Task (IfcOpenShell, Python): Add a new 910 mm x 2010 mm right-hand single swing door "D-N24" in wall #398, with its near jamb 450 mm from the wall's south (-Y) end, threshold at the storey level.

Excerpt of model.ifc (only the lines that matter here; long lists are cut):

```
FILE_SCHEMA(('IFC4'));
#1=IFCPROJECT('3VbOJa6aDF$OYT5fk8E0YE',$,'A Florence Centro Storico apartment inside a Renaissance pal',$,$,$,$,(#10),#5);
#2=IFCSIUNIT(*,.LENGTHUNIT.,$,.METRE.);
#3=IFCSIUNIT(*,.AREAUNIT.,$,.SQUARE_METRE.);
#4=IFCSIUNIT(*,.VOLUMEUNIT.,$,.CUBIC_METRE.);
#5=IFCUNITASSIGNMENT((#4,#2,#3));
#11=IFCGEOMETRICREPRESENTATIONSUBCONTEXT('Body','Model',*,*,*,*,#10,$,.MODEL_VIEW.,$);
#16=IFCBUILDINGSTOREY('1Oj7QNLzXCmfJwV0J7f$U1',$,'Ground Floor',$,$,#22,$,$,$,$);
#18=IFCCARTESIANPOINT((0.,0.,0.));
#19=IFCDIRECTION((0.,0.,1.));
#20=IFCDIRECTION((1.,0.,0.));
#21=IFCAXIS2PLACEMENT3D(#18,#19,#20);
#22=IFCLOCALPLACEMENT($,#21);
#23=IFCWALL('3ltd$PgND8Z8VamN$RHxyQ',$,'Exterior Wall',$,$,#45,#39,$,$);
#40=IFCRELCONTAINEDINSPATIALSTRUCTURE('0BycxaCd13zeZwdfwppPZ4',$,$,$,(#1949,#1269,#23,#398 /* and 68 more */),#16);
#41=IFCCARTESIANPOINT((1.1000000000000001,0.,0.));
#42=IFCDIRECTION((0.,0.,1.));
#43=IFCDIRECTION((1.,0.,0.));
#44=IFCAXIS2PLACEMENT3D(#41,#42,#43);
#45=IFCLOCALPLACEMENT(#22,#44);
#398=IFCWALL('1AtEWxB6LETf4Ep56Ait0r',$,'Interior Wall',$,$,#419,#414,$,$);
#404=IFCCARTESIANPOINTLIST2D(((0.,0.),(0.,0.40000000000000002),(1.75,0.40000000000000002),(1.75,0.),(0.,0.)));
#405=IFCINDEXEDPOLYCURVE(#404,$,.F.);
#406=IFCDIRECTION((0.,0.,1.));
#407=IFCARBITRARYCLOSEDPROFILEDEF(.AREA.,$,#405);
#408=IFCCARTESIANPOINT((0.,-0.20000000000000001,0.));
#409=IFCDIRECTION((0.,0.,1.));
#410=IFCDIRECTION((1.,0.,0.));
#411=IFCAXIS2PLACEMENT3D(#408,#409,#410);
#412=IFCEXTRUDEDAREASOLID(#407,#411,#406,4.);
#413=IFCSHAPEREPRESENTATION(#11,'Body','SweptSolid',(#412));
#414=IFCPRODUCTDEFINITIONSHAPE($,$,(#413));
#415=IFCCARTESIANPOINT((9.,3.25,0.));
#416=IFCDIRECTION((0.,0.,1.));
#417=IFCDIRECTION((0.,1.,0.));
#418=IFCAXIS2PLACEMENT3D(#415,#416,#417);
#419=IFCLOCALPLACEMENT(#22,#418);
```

```python
import numpy as np
import ifcopenshell
import ifcopenshell.api.feature
import ifcopenshell.api.geometry
import ifcopenshell.api.root
import ifcopenshell.api.spatial
import ifcopenshell.geom
import ifcopenshell.util.element
import ifcopenshell.util.placement
import ifcopenshell.util.representation
import ifcopenshell.util.shape
import ifcopenshell.util.unit

model = ifcopenshell.open("model.ifc")
unit_scale = ifcopenshell.util.unit.calculate_unit_scale(model)
settings = ifcopenshell.geom.settings()


def volume(element):
    """Net volume in cubic metres, openings subtracted."""
    shape = ifcopenshell.geom.create_shape(settings, element)
    return ifcopenshell.util.shape.get_volume(shape.geometry)


wall = model.by_guid("1AtEWxB6LETf4Ep56Ait0r")
storey = ifcopenshell.util.element.get_container(wall, ifc_class="IfcBuildingStorey")
context = ifcopenshell.util.representation.get_context(model, "Model", "Body", "MODEL_VIEW")
before = volume(wall)

width, height, from_end, sill = 0.91, 2.01, 0.45, 0.0  # metres

# The wall runs along its own X axis, and the end named is its -X end.
wall_shape = ifcopenshell.geom.create_shape(settings, wall)
x, y, z = ifcopenshell.util.shape.get_vertices(wall_shape.geometry).T
start = x.min() + from_end
face, thickness = float(y.min()), float(y.max() - y.min())
wall_matrix = ifcopenshell.util.placement.get_local_placement(wall.ObjectPlacement)
level = ifcopenshell.util.placement.get_local_placement(storey.ObjectPlacement)[2, 3]


def in_wall(x, y):
    """Placement at x, y metres in the wall's axes, at sill height."""
    matrix = wall_matrix.copy()
    matrix[:, 3] = wall_matrix @ np.array([x / unit_scale, y / unit_scale, 0.0, 1.0])
    matrix[2, 3] = level + sill / unit_scale
    return matrix


# Opening: a box that overshoots both wall faces by 50 mm.
opening = ifcopenshell.api.root.create_entity(model, ifc_class="IfcOpeningElement", predefined_type="OPENING")
box = ifcopenshell.api.geometry.add_wall_representation(
    model, context=context, length=width, height=height, thickness=thickness + 0.1
)
ifcopenshell.api.geometry.assign_representation(model, product=opening, representation=box)
ifcopenshell.api.geometry.edit_object_placement(model, product=opening, matrix=in_wall(start, face - 0.05), is_si=False)
ifcopenshell.api.feature.add_feature(model, feature=opening, element=wall)

door = ifcopenshell.api.root.create_entity(model, ifc_class="IfcDoor", name="D-N24", predefined_type="DOOR")
door.OverallWidth, door.OverallHeight = width / unit_scale, height / unit_scale
door.OperationType = "SINGLE_SWING_RIGHT"
body = ifcopenshell.api.geometry.add_door_representation(
    model,
    context=context,
    overall_width=door.OverallWidth,
    overall_height=door.OverallHeight,
    operation_type="SINGLE_SWING_RIGHT",
    lining_properties={"LiningDepth": thickness / unit_scale, "ThresholdDepth": thickness / unit_scale},
)
ifcopenshell.api.geometry.assign_representation(model, product=door, representation=body)
ifcopenshell.api.spatial.assign_container(model, products=[door], relating_structure=storey)
ifcopenshell.api.feature.add_filling(model, opening=opening, element=door)

# The lining spans the wall, so the door starts at the wall face.
ifcopenshell.api.geometry.edit_object_placement(model, product=door, matrix=in_wall(start, face), is_si=False)

after = volume(wall)

print(f"wall volume {before:.3f} -> {after:.3f} m3")

model.write("model_edited.ifc")
```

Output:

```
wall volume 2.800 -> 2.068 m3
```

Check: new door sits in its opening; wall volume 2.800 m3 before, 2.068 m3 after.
